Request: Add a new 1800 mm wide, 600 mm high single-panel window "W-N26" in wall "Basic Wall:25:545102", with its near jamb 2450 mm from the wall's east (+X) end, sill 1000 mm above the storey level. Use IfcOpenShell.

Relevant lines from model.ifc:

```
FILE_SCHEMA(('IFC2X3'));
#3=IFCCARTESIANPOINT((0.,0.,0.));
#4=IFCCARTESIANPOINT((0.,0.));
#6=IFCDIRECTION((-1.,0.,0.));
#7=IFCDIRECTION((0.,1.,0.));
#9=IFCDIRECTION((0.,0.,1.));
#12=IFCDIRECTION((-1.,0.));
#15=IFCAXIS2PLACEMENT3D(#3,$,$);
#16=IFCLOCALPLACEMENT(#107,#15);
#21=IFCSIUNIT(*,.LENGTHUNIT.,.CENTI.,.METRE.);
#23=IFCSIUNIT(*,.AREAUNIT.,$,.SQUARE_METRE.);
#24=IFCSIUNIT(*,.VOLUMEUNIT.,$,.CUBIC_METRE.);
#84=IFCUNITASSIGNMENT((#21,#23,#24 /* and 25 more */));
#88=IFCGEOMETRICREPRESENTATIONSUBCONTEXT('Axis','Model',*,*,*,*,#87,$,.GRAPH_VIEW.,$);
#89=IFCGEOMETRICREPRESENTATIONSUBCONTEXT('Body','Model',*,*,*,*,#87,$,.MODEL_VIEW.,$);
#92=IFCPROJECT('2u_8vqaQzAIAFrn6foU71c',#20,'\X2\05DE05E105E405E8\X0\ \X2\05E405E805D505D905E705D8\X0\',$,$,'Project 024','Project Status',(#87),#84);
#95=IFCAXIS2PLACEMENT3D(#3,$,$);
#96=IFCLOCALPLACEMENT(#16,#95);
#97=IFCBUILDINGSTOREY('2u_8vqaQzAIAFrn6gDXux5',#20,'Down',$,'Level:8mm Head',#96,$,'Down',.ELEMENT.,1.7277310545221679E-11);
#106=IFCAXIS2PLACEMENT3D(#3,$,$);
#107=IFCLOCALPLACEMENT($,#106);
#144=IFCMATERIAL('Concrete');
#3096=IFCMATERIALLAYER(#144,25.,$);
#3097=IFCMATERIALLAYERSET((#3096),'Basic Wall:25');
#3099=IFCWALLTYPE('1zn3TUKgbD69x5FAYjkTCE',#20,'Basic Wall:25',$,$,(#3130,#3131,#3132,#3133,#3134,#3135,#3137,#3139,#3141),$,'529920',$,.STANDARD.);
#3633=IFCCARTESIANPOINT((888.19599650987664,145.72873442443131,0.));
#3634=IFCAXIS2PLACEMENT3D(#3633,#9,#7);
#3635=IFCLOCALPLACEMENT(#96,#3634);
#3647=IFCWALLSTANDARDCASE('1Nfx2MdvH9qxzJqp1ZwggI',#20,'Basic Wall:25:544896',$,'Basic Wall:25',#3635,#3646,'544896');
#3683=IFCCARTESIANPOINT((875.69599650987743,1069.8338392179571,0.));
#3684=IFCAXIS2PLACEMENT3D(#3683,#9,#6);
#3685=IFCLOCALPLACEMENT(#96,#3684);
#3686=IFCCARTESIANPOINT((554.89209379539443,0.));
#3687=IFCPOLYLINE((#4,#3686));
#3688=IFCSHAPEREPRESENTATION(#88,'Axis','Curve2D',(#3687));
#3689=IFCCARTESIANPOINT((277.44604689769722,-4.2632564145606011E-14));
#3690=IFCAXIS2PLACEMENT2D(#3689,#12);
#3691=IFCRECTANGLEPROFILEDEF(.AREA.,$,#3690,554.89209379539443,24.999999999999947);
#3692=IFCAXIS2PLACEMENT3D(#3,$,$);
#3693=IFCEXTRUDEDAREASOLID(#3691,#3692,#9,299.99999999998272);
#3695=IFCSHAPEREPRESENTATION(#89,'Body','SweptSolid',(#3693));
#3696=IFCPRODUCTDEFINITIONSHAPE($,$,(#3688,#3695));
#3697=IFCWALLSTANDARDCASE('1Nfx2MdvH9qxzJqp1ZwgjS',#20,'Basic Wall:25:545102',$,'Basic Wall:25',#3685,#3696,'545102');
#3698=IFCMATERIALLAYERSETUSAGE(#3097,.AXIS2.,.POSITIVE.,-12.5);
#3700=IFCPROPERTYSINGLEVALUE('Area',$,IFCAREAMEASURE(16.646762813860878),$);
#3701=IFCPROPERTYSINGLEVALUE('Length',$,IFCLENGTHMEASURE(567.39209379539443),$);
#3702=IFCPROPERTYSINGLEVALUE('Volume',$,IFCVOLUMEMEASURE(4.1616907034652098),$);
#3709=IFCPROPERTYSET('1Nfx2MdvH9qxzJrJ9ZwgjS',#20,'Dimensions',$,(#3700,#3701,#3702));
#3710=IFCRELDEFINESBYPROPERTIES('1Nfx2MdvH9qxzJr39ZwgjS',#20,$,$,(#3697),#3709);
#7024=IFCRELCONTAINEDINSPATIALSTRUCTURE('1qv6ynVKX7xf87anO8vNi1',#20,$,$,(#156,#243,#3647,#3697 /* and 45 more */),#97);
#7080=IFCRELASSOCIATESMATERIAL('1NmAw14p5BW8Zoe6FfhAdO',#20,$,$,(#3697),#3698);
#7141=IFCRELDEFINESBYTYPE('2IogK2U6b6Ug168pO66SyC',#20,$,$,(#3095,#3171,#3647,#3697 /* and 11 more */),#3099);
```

```python
import numpy as np
import ifcopenshell
import ifcopenshell.api.feature
import ifcopenshell.api.geometry
import ifcopenshell.api.pset
import ifcopenshell.api.root
import ifcopenshell.api.spatial
import ifcopenshell.api.type
import ifcopenshell.geom
import ifcopenshell.util.element
import ifcopenshell.util.placement
import ifcopenshell.util.representation
import ifcopenshell.util.shape
import ifcopenshell.util.unit

model = ifcopenshell.open("model.ifc")
unit_scale = ifcopenshell.util.unit.calculate_unit_scale(model)
area_scale = ifcopenshell.util.unit.calculate_unit_scale(model, "AREAUNIT")
volume_scale = ifcopenshell.util.unit.calculate_unit_scale(model, "VOLUMEUNIT")
settings = ifcopenshell.geom.settings()


def volume(element):
    """Net volume in cubic metres, openings subtracted."""
    shape = ifcopenshell.geom.create_shape(settings, element)
    return ifcopenshell.util.shape.get_volume(shape.geometry)


wall = model.by_guid("1Nfx2MdvH9qxzJqp1ZwgjS")
storey = ifcopenshell.util.element.get_container(wall, ifc_class="IfcBuildingStorey")
context = ifcopenshell.util.representation.get_context(model, "Model", "Body", "MODEL_VIEW")
before = volume(wall)

width, height, from_end, sill = 1.8, 0.6, 2.45, 1  # metres

# The wall runs along its own X axis, and the end named is its -X end.
wall_shape = ifcopenshell.geom.create_shape(settings, wall)
x, y, z = ifcopenshell.util.shape.get_vertices(wall_shape.geometry).T
start = x.min() + from_end
face, thickness = float(y.min()), float(y.max() - y.min())
wall_matrix = ifcopenshell.util.placement.get_local_placement(wall.ObjectPlacement)
level = ifcopenshell.util.placement.get_local_placement(storey.ObjectPlacement)[2, 3]


def in_wall(x, y):
    """Placement at x, y metres in the wall's axes, at sill height."""
    matrix = wall_matrix.copy()
    matrix[:, 3] = wall_matrix @ np.array([x / unit_scale, y / unit_scale, 0.0, 1.0])
    matrix[2, 3] = level + sill / unit_scale
    return matrix


# Opening: a box that overshoots both wall faces by 50 mm.
opening = ifcopenshell.api.root.create_entity(model, ifc_class="IfcOpeningElement")
box = ifcopenshell.api.geometry.add_wall_representation(
    model, context=context, length=width, height=height, thickness=thickness + 0.1
)
ifcopenshell.api.geometry.assign_representation(model, product=opening, representation=box)
ifcopenshell.api.geometry.edit_object_placement(model, product=opening, matrix=in_wall(start, face - 0.05), is_si=False)
ifcopenshell.api.feature.add_feature(model, feature=opening, element=wall)

window = ifcopenshell.api.root.create_entity(model, ifc_class="IfcWindow", name="W-N26")
window.OverallWidth, window.OverallHeight = width / unit_scale, height / unit_scale
body = ifcopenshell.api.geometry.add_window_representation(
    model,
    context=context,
    overall_width=window.OverallWidth,
    overall_height=window.OverallHeight,
    partition_type="SINGLE_PANEL",
)
ifcopenshell.api.geometry.assign_representation(model, product=window, representation=body)
ifcopenshell.api.spatial.assign_container(model, products=[window], relating_structure=storey)
fills = ifcopenshell.api.feature.add_filling(model, opening=opening, element=window)
fills.OwnerHistory = window.OwnerHistory  # required in IFC2X3

# IFC2X3 keeps the operation on the window style.
style = ifcopenshell.api.root.create_entity(model, ifc_class="IfcWindowStyle", name="W-N26")
style.OperationType, style.ConstructionType = "SINGLE_PANEL", "NOTDEFINED"
style.ParameterTakesPrecedence = style.Sizeable = False
ifcopenshell.api.type.assign_type(model, related_objects=[window], relating_type=style)

# Centre the window in the wall's thickness.
ifcopenshell.api.geometry.edit_object_placement(model, product=window, matrix=in_wall(start, face), is_si=False)
window_shape = ifcopenshell.geom.create_shape(settings, window)
depth = ifcopenshell.util.shape.get_vertices(window_shape.geometry)[:, 1]
offset = face + thickness / 2 - (depth.min() + depth.max()) / 2
ifcopenshell.api.geometry.edit_object_placement(model, product=window, matrix=in_wall(start, offset), is_si=False)

after = volume(wall)

# Update the wall's stored quantities.
pset = model.by_id(ifcopenshell.util.element.get_pset(wall, "Dimensions", should_inherit=False)["id"])
ifcopenshell.api.pset.edit_pset(model, pset=pset, properties={
    "Area": model.create_entity("IfcAreaMeasure", after / thickness / area_scale),
    "Volume": model.create_entity("IfcVolumeMeasure", after / volume_scale),
})

print(f"wall volume {before:.3f} -> {after:.3f} m3")

model.write("model_edited.ifc")
```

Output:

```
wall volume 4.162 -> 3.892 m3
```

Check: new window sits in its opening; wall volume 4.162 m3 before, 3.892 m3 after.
